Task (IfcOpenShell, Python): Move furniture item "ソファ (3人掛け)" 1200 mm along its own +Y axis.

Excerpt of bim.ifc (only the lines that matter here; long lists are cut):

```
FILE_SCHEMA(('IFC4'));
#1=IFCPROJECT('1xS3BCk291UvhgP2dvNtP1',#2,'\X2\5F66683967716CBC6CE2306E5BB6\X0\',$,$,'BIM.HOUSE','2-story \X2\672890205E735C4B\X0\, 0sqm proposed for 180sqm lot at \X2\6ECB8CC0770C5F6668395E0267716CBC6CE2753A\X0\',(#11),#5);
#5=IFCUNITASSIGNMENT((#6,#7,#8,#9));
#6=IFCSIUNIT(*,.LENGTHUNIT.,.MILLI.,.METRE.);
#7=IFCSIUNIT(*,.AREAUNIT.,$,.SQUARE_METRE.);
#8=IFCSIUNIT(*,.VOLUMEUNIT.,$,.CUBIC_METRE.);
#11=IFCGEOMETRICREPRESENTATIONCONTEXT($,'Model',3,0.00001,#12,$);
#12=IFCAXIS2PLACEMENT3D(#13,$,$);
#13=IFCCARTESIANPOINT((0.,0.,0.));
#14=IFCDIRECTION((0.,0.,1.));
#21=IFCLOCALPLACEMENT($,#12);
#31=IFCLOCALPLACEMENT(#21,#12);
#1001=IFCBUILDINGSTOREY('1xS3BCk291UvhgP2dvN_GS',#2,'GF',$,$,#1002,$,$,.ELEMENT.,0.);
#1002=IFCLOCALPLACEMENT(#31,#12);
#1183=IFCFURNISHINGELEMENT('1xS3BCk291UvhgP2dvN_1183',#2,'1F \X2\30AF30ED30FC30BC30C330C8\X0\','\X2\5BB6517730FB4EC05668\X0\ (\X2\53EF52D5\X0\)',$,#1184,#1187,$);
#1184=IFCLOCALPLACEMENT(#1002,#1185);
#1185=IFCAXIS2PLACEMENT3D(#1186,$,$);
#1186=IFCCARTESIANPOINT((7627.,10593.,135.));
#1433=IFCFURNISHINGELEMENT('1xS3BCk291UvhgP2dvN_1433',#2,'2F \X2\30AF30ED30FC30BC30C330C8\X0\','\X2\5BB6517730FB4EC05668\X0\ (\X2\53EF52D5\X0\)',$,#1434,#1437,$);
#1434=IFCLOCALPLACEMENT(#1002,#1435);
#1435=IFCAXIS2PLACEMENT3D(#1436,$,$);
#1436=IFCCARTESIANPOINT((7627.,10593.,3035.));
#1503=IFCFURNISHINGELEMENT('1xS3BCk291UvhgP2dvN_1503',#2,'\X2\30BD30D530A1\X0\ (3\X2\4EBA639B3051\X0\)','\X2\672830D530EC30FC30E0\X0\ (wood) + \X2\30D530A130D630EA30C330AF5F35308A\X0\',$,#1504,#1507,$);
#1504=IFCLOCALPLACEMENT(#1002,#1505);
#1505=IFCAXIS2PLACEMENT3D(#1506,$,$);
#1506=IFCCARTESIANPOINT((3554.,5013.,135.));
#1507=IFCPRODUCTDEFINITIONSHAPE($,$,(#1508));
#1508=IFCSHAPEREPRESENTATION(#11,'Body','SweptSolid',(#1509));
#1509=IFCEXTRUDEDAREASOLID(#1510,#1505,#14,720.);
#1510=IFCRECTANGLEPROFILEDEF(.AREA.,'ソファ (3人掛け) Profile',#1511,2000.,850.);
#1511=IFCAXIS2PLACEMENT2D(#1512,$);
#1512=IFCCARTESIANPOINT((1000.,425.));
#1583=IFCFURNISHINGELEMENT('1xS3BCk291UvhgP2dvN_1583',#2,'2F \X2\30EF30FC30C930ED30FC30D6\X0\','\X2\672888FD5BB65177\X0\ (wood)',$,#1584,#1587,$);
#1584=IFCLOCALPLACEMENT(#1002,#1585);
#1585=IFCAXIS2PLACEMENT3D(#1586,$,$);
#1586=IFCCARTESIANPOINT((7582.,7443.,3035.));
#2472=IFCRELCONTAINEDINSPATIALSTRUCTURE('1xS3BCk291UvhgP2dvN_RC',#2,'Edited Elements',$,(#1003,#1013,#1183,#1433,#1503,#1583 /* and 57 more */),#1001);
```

```python
import ifcopenshell
import ifcopenshell.api.geometry
import ifcopenshell.util.placement

model = ifcopenshell.open("bim.ifc")

item = model.by_guid("1xS3BCk291UvhgP2dvN_1503")
matrix = ifcopenshell.util.placement.get_local_placement(item.ObjectPlacement)
matrix[:3, 3] += matrix[:3, 1] * 1200.0
ifcopenshell.api.geometry.edit_object_placement(model, product=item, matrix=matrix, is_si=False)

print(ifcopenshell.util.placement.get_local_placement(item.ObjectPlacement).round(3) + 0.0)

model.write("bim_edited.ifc")
```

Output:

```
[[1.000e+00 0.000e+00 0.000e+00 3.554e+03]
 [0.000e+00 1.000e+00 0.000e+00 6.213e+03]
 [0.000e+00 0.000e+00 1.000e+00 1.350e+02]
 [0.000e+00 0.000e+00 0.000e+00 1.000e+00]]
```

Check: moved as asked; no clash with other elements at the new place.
